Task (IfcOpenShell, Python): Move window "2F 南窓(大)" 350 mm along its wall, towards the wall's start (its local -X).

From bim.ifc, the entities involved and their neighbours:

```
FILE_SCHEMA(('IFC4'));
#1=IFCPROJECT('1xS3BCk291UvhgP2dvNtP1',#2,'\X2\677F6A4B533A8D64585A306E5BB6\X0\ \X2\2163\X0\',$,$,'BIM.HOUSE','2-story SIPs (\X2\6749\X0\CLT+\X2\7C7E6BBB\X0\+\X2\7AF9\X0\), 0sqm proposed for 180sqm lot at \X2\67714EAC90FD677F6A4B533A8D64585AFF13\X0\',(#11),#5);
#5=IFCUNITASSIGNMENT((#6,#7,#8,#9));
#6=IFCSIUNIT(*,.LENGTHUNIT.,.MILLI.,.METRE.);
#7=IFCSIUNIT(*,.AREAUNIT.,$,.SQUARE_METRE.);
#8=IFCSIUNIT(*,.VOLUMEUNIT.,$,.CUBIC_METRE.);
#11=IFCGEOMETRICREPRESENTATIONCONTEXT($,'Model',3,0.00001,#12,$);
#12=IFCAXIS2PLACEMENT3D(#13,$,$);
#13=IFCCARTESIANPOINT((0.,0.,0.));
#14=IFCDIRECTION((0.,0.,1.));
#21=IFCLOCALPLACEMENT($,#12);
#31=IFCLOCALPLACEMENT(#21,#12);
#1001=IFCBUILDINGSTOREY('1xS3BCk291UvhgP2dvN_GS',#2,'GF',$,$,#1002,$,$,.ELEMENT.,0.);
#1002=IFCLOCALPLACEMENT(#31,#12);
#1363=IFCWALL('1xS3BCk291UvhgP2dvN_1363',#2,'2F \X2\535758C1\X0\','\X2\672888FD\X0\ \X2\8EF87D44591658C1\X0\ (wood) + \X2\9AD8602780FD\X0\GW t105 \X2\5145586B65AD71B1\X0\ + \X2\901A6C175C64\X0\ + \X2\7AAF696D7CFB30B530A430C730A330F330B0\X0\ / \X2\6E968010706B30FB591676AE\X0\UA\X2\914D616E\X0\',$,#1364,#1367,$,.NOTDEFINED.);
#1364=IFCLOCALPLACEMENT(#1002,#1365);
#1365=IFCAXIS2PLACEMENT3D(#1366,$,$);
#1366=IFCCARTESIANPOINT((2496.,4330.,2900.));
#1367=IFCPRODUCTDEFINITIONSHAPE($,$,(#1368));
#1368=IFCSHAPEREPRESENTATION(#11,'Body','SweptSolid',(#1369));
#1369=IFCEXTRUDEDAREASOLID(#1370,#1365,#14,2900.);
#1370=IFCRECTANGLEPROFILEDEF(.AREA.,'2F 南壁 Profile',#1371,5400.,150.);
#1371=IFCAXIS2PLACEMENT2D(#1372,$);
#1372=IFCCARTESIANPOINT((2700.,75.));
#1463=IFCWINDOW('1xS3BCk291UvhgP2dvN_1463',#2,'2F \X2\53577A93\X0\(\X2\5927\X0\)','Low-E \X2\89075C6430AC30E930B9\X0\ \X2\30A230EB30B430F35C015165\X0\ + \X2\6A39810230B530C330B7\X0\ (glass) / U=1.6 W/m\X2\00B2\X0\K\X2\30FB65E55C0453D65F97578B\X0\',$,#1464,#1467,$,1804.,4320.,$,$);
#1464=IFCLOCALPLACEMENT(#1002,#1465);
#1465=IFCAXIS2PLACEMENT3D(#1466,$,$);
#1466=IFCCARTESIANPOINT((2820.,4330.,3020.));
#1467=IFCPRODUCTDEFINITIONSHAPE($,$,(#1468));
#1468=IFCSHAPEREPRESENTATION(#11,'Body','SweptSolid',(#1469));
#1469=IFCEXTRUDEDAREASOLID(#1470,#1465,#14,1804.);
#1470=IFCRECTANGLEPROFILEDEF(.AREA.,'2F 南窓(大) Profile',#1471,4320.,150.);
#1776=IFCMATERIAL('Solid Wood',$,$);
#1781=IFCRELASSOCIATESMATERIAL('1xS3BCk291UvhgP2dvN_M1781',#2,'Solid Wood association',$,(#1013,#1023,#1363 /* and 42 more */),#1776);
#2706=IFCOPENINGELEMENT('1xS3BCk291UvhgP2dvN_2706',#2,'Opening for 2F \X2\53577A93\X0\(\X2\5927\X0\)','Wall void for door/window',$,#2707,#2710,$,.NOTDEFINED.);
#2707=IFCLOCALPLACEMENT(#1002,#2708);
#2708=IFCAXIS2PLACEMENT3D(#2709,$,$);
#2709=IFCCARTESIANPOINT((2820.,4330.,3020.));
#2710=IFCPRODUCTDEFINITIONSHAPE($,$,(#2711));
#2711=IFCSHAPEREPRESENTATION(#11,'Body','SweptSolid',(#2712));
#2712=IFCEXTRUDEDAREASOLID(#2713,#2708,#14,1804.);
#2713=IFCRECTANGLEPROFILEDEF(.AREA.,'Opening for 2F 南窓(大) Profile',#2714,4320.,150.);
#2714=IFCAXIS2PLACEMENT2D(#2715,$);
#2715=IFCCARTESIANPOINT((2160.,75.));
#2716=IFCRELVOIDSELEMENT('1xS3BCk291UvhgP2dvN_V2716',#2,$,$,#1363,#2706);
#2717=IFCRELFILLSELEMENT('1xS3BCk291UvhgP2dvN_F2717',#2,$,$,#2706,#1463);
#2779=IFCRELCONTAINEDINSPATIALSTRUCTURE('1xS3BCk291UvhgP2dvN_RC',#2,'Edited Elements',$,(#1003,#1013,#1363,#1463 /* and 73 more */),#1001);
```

```python
import ifcopenshell
import ifcopenshell.api.geometry
import ifcopenshell.util.placement

model = ifcopenshell.open("bim.ifc")

window = model.by_guid("1xS3BCk291UvhgP2dvN_1463")
opening = window.FillsVoids[0].RelatingOpeningElement
wall = opening.VoidsElements[0].RelatingBuildingElement

wall_matrix = ifcopenshell.util.placement.get_local_placement(wall.ObjectPlacement)
shift = wall_matrix[:3, 0] * -350.0
before = ifcopenshell.util.placement.get_local_placement(window.ObjectPlacement)[:3, 3].copy()

# The window is not placed relative to its opening, so move both.
for product in (opening, window):
    matrix = ifcopenshell.util.placement.get_local_placement(product.ObjectPlacement)
    matrix[:3, 3] += shift
    ifcopenshell.api.geometry.edit_object_placement(model, product=product, matrix=matrix, is_si=False)

after = ifcopenshell.util.placement.get_local_placement(window.ObjectPlacement)[:3, 3]
print("window moved by", (after - before).round(3) + 0.0)

model.write("bim_updated.ifc")
```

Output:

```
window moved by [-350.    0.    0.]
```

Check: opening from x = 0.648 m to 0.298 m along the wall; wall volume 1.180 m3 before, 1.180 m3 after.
